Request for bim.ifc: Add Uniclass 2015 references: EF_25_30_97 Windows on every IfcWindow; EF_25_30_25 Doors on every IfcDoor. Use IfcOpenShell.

First a look at what the model holds.

```python
import ifcopenshell

model = ifcopenshell.open("bim.ifc")
print(model.schema)
print("classifications:", [c.Name for c in model.by_type("IfcClassification")])
for ifc_class in ("IfcDoor", "IfcRoof", "IfcStair", "IfcWall", "IfcWindow"):
    print(ifc_class, len(model.by_type(ifc_class)))
```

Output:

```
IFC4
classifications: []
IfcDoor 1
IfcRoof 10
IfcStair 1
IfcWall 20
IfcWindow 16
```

```python
import ifcopenshell
import ifcopenshell.api.classification

model = ifcopenshell.open("bim.ifc")

system = ifcopenshell.api.classification.add_classification(model, classification="Uniclass 2015")

codes = {
    "IfcWindow": ("EF_25_30_97", "Windows"),
    "IfcDoor": ("EF_25_30_25", "Doors"),
}
for ifc_class, (code, name) in codes.items():
    products = model.by_type(ifc_class)
    ifcopenshell.api.classification.add_reference(
        model, products=products, classification=system, identification=code, name=name
    )
    print(code, len(products))

model.write("bim-out.ifc")
```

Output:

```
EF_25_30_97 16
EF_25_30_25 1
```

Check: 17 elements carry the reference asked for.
